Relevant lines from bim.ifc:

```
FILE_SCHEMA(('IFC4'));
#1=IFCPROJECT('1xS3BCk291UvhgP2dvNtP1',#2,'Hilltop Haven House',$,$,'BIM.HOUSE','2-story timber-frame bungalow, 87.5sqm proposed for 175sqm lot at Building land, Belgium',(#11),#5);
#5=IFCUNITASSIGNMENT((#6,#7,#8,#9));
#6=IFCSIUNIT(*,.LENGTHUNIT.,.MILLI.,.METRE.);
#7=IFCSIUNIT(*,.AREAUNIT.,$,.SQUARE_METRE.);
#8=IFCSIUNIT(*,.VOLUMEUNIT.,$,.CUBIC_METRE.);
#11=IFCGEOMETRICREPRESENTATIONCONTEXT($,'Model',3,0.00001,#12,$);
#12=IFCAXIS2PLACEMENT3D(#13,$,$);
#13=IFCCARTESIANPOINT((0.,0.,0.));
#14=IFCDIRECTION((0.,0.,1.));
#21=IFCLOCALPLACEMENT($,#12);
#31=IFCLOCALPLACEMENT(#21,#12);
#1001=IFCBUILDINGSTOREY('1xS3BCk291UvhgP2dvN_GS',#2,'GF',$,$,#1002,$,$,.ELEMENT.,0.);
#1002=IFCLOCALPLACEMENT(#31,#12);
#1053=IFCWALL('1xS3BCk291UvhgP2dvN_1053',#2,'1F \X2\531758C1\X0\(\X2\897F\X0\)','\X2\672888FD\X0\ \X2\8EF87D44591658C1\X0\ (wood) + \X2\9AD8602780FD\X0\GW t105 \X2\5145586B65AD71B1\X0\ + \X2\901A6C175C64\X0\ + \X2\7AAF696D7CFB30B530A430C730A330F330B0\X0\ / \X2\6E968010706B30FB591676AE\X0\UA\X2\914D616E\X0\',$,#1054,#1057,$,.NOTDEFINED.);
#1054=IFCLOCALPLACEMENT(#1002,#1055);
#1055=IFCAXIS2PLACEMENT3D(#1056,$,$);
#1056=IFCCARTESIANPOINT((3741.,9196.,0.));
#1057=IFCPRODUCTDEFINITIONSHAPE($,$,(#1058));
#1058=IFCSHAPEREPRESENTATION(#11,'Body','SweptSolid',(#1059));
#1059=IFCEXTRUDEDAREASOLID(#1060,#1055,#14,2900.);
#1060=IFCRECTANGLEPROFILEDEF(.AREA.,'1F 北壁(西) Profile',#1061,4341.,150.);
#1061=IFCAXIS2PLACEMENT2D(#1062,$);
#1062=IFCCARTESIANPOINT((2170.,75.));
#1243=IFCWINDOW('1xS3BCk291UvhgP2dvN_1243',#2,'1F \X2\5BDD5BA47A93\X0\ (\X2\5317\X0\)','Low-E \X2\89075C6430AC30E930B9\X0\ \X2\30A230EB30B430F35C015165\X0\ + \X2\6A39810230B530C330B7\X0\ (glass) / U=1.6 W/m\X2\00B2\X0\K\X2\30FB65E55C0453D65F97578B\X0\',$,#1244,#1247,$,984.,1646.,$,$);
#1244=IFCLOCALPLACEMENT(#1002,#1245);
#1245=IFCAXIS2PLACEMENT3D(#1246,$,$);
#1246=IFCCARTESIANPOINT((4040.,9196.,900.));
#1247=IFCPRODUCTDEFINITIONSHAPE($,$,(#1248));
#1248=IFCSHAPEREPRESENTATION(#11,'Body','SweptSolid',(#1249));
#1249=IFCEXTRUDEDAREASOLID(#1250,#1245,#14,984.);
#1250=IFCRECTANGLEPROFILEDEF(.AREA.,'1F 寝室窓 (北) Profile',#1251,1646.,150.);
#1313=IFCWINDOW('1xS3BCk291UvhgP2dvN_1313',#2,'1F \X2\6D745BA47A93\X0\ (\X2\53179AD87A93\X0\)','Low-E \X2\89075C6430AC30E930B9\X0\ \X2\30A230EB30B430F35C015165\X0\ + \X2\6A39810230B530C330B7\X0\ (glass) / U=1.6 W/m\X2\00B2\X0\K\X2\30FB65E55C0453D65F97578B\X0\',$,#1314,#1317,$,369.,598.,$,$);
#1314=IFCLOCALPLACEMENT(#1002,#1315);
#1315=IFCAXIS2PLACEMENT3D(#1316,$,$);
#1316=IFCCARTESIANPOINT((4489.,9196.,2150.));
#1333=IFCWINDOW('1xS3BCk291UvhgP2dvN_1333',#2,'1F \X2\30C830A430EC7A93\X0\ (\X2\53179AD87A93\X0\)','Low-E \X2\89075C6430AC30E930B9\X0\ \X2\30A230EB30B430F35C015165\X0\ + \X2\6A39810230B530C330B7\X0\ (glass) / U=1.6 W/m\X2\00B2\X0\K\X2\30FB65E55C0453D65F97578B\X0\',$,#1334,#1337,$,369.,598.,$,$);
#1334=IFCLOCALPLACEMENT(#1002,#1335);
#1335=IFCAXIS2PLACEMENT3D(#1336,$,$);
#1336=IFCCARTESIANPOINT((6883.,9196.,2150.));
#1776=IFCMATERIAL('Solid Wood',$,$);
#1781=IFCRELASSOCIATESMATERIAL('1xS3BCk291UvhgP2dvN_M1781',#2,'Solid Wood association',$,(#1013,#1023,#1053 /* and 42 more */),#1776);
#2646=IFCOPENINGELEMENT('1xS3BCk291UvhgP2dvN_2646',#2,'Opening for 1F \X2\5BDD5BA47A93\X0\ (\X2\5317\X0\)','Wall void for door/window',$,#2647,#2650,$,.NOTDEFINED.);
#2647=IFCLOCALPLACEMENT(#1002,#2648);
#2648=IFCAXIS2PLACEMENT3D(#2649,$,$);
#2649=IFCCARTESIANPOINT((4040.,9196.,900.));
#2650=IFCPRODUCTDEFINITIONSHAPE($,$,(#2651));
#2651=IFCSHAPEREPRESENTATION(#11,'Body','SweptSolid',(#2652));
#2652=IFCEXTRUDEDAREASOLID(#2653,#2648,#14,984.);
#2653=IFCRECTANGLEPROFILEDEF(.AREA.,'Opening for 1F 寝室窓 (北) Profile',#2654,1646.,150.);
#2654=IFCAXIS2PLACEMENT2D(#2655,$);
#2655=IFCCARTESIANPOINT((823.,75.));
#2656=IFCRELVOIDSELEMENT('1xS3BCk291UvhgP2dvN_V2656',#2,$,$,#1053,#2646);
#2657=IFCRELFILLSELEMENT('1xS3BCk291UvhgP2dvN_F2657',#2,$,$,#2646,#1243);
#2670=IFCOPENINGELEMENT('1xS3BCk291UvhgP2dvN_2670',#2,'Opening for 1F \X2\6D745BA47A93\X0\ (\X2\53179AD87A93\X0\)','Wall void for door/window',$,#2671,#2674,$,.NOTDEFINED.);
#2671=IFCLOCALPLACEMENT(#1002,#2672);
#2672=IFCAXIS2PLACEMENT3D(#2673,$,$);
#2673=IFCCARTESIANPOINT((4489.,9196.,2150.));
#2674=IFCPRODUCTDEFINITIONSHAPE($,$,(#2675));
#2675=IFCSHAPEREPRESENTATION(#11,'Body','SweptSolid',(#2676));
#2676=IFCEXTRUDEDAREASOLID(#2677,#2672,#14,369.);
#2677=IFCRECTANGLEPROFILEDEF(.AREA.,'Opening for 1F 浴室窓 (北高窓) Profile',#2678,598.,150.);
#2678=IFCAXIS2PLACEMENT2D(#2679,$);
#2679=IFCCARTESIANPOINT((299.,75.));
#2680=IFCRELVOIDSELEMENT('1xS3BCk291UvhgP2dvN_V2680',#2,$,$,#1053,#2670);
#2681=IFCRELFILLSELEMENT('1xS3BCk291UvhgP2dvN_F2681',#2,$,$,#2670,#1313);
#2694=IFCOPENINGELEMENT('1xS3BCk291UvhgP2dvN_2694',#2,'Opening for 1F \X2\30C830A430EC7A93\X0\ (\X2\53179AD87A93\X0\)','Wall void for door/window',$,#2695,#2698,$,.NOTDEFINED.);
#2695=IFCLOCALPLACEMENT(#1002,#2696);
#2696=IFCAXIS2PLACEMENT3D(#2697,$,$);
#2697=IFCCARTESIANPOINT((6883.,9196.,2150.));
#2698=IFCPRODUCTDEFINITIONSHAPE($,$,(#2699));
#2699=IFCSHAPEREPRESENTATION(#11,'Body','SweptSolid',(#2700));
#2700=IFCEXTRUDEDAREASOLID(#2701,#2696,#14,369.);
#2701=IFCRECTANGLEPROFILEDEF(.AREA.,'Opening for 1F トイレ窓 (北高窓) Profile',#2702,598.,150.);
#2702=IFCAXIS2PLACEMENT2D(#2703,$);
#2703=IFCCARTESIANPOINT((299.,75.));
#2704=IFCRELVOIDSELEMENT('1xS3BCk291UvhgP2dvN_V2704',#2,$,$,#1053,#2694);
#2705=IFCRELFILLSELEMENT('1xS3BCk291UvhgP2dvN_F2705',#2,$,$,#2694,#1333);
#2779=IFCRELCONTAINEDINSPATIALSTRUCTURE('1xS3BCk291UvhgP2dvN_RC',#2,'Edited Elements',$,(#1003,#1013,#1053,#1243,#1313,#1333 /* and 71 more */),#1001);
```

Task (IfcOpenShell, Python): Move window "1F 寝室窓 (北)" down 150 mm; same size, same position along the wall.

```python
import numpy as np
import ifcopenshell
import ifcopenshell.api.geometry
import ifcopenshell.util.placement
import ifcopenshell.util.unit

model = ifcopenshell.open("bim.ifc")
unit_scale = ifcopenshell.util.unit.calculate_unit_scale(model)

window = model.by_guid("1xS3BCk291UvhgP2dvN_1243")
opening = window.FillsVoids[0].RelatingOpeningElement
dz = -150.0

shift = np.array([0.0, 0.0, dz])
# The window is not placed relative to its opening, so move both.
for product in (opening, window):
    matrix = ifcopenshell.util.placement.get_local_placement(product.ObjectPlacement)
    matrix[:3, 3] += shift
    ifcopenshell.api.geometry.edit_object_placement(model, product=product, matrix=matrix, is_si=False)

print(f"moved by {dz * unit_scale:+.3f} m")

model.write("bim_edited.ifc")
```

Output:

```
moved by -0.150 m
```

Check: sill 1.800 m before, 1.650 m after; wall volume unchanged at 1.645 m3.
